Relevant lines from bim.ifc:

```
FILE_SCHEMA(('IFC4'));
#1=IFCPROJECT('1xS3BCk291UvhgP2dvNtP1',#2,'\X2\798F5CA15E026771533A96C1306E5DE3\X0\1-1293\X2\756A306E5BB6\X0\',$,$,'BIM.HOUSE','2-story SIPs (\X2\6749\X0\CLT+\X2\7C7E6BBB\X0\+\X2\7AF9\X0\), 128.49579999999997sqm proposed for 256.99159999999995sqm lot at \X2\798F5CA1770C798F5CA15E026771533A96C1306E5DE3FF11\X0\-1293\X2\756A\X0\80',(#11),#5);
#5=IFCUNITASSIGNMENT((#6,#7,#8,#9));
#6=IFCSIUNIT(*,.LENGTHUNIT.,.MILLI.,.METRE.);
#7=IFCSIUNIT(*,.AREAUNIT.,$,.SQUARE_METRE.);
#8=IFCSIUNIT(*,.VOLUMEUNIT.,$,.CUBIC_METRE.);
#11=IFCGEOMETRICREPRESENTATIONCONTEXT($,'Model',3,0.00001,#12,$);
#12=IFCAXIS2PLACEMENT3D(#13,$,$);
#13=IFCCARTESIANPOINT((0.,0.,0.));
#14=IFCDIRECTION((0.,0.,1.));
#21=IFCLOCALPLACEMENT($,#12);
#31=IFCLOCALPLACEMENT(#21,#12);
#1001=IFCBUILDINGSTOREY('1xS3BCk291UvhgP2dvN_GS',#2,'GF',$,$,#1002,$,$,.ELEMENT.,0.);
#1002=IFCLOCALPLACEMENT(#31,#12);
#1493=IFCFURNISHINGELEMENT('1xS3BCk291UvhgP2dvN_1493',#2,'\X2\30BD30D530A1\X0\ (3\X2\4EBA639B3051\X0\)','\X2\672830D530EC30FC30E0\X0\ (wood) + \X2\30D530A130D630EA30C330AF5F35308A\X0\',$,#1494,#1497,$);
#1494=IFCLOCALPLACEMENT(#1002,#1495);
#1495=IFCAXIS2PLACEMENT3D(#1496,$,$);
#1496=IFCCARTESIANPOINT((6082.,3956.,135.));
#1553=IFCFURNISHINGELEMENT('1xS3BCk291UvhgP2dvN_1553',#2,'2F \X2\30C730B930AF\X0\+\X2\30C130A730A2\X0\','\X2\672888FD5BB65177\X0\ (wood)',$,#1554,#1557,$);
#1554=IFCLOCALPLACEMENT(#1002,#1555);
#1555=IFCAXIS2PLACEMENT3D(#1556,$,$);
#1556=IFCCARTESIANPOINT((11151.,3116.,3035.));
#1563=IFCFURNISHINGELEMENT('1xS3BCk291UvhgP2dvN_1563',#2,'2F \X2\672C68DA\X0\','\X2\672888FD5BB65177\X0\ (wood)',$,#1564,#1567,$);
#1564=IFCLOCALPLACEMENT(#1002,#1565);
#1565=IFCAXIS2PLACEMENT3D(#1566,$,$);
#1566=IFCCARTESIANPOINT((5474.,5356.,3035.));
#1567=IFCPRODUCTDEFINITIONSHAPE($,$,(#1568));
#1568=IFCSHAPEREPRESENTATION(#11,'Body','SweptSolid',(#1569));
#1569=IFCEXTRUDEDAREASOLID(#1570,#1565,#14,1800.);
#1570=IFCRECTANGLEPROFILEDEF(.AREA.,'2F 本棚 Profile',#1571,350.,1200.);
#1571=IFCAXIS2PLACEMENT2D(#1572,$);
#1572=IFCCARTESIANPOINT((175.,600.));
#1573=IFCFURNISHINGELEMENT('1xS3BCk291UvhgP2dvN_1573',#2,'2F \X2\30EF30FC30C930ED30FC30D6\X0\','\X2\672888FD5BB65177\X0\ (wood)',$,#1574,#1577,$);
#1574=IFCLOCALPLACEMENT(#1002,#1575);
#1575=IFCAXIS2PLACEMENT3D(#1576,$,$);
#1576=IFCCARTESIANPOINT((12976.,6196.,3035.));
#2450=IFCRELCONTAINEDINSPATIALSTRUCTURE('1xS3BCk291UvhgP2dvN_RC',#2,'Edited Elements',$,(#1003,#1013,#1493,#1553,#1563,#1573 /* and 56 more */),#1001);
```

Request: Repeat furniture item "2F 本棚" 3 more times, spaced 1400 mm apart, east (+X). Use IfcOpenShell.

```python
import numpy as np
import ifcopenshell
import ifcopenshell.api.geometry
import ifcopenshell.api.root
import ifcopenshell.util.element
import ifcopenshell.util.placement
import ifcopenshell.util.unit

model = ifcopenshell.open("bim.ifc")
unit_scale = ifcopenshell.util.unit.calculate_unit_scale(model)


def reuse_history(source, copy):
    """copy_class also copies each property set's owner history, people and application; keep the originals."""
    for rel in copy.IsDefinedBy:
        if rel.is_a("IfcRelDefinesByProperties") and (history := rel.RelatingPropertyDefinition.OwnerHistory):
            rel.RelatingPropertyDefinition.OwnerHistory = source.OwnerHistory
            ifcopenshell.util.element.remove_deep2(model, history)


source = model.by_guid("1xS3BCk291UvhgP2dvN_1563")
base = ifcopenshell.util.placement.get_local_placement(source.ObjectPlacement)
step = np.array([1.0, 0.0, 0.0]) * 1.4 / unit_scale

for i in range(1, 4):
    copy = ifcopenshell.api.root.copy_class(model, product=source)
    copy.Representation = ifcopenshell.util.element.copy_deep(
        model, source.Representation, exclude=["IfcGeometricRepresentationContext", "IfcRepresentationMap"]
    )
    reuse_history(source, copy)
    matrix = base.copy()
    matrix[:3, 3] += i * step
    print("added at", matrix[:3, 3].round(3) + 0.0)
    ifcopenshell.api.geometry.edit_object_placement(model, product=copy, matrix=matrix, is_si=False)

model.write("bim_edited.ifc")
```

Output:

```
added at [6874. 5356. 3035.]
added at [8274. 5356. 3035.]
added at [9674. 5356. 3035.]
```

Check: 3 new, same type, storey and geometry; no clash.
